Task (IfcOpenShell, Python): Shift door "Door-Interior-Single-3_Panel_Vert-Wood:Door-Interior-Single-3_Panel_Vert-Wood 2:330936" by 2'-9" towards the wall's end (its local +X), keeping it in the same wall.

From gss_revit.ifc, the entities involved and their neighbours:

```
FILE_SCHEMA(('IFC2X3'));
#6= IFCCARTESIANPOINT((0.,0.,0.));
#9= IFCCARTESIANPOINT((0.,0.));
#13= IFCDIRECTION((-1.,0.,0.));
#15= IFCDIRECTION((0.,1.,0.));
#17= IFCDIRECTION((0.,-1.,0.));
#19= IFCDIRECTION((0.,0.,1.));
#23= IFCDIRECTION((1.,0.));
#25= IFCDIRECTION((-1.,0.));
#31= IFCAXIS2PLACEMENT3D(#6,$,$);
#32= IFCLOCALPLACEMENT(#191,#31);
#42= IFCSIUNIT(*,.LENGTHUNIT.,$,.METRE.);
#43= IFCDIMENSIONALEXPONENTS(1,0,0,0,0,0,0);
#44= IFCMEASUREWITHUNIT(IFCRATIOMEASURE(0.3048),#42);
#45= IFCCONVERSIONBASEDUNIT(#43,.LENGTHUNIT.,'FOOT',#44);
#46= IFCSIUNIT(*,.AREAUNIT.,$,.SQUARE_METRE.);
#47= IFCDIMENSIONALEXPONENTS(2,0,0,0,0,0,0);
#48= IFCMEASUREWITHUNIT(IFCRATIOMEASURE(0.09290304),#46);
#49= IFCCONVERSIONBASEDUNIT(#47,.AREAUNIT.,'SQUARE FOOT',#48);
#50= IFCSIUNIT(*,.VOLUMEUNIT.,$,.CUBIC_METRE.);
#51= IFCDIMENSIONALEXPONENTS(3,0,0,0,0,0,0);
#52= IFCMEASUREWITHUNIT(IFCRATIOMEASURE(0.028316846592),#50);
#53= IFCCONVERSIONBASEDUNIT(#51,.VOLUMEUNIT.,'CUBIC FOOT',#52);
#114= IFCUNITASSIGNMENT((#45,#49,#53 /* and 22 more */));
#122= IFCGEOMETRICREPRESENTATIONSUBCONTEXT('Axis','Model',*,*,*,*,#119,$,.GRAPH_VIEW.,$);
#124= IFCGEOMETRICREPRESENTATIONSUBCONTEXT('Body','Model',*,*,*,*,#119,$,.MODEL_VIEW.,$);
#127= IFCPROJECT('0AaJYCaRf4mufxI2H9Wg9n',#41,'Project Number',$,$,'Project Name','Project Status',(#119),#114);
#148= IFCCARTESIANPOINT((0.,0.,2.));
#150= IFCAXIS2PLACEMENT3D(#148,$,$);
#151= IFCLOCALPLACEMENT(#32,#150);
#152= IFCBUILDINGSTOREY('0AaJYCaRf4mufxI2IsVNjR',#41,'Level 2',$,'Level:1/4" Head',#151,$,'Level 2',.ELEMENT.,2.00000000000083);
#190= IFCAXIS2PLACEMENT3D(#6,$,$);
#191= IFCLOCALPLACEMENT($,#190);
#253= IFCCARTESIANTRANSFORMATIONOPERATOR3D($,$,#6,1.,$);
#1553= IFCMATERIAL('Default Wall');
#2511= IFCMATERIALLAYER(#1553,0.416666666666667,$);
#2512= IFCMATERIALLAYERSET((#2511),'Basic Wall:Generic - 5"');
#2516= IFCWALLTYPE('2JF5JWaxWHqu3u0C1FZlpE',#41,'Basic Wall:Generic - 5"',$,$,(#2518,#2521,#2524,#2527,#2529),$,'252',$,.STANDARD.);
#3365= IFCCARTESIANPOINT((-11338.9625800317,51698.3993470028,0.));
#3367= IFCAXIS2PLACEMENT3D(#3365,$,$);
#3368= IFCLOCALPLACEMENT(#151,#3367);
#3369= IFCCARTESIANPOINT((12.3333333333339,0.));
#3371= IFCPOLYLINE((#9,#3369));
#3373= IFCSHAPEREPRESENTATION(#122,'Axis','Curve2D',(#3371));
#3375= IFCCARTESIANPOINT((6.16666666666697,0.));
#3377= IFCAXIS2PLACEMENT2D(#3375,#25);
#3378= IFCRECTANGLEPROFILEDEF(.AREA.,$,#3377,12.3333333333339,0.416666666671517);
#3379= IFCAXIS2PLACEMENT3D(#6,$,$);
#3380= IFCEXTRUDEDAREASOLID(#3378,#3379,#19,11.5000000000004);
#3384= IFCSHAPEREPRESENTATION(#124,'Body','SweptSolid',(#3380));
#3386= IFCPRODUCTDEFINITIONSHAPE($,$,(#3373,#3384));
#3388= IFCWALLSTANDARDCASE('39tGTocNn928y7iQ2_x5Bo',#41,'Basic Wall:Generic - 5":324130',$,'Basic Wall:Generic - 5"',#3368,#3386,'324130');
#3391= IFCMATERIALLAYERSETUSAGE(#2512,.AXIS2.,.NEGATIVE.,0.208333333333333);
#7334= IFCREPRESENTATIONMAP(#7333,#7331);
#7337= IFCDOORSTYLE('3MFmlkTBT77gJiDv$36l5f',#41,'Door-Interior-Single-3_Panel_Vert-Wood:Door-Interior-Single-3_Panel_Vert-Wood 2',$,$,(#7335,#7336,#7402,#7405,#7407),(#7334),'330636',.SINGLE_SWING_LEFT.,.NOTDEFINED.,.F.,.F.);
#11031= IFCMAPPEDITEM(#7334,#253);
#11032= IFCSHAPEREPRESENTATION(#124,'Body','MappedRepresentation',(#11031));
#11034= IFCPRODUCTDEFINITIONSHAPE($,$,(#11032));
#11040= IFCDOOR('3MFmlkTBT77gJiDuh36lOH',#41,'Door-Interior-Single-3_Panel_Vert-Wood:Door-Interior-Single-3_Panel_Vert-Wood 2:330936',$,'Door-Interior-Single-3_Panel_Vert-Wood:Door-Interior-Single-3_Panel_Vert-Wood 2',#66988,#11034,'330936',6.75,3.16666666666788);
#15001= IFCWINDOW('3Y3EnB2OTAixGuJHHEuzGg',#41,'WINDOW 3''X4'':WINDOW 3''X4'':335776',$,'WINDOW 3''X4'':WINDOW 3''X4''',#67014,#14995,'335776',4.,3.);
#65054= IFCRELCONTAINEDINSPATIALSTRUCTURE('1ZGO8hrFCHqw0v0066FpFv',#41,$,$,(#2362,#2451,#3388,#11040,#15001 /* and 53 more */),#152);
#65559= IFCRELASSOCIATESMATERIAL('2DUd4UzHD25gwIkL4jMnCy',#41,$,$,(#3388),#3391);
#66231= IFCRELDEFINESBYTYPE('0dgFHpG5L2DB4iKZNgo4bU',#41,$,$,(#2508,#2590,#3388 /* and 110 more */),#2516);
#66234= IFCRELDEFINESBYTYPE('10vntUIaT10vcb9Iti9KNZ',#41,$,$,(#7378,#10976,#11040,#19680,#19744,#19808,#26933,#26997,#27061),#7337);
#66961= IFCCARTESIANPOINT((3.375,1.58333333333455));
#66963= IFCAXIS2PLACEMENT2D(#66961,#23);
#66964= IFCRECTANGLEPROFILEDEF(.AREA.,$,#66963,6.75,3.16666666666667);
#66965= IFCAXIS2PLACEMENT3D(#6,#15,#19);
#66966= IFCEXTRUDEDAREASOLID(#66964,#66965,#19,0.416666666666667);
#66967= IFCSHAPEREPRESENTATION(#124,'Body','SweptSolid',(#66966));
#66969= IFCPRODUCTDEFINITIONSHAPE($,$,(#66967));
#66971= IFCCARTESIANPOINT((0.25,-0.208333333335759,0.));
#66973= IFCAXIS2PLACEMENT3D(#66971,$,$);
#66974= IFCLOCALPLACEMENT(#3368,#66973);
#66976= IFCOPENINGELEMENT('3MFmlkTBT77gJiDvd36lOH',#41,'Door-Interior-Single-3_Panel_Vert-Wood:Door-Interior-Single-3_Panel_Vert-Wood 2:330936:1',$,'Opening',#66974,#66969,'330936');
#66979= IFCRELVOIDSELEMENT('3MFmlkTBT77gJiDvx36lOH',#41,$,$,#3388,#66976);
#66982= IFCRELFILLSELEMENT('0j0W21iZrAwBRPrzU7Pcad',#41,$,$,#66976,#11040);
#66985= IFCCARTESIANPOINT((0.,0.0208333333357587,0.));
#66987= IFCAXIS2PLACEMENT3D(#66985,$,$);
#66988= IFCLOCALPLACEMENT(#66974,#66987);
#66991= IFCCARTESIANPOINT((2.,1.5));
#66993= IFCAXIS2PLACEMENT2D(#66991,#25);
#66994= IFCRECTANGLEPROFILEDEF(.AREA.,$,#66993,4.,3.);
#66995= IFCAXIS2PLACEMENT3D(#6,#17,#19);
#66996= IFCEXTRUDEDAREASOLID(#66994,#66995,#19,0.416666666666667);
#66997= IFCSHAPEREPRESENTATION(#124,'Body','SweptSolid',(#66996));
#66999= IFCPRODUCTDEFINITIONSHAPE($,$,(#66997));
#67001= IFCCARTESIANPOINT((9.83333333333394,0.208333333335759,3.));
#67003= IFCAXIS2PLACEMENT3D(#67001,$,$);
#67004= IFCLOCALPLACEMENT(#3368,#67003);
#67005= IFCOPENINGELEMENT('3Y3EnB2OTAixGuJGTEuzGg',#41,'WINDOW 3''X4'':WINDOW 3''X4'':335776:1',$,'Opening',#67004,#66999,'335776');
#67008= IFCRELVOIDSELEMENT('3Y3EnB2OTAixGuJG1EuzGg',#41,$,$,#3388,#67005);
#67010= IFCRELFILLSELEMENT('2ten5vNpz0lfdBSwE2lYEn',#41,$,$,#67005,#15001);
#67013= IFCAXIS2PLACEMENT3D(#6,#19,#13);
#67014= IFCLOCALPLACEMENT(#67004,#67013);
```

```python
import ifcopenshell
import ifcopenshell.api.geometry
import ifcopenshell.util.placement
import ifcopenshell.util.unit

model = ifcopenshell.open("gss_revit.ifc")
unit_scale = ifcopenshell.util.unit.calculate_unit_scale(model)

door = model.by_id(11040)
opening = door.FillsVoids[0].RelatingOpeningElement
wall = opening.VoidsElements[0].RelatingBuildingElement

wall_matrix = ifcopenshell.util.placement.get_local_placement(wall.ObjectPlacement)
shift = wall_matrix[:3, 0] * 33 * 0.0254 / unit_scale
before = ifcopenshell.util.placement.get_local_placement(door.ObjectPlacement)[:3, 3].copy()

# The door is placed relative to its opening, so it follows when the opening moves.
matrix = ifcopenshell.util.placement.get_local_placement(opening.ObjectPlacement)
matrix[:3, 3] += shift
ifcopenshell.api.geometry.edit_object_placement(
    model, product=opening, matrix=matrix, is_si=False, should_transform_children=True
)

after = ifcopenshell.util.placement.get_local_placement(door.ObjectPlacement)[:3, 3]
print("door moved by", (after - before).round(3) + 0.0)

model.write("gss_revit_v2.ifc")
```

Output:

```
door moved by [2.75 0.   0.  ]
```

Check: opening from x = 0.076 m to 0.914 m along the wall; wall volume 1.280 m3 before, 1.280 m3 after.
